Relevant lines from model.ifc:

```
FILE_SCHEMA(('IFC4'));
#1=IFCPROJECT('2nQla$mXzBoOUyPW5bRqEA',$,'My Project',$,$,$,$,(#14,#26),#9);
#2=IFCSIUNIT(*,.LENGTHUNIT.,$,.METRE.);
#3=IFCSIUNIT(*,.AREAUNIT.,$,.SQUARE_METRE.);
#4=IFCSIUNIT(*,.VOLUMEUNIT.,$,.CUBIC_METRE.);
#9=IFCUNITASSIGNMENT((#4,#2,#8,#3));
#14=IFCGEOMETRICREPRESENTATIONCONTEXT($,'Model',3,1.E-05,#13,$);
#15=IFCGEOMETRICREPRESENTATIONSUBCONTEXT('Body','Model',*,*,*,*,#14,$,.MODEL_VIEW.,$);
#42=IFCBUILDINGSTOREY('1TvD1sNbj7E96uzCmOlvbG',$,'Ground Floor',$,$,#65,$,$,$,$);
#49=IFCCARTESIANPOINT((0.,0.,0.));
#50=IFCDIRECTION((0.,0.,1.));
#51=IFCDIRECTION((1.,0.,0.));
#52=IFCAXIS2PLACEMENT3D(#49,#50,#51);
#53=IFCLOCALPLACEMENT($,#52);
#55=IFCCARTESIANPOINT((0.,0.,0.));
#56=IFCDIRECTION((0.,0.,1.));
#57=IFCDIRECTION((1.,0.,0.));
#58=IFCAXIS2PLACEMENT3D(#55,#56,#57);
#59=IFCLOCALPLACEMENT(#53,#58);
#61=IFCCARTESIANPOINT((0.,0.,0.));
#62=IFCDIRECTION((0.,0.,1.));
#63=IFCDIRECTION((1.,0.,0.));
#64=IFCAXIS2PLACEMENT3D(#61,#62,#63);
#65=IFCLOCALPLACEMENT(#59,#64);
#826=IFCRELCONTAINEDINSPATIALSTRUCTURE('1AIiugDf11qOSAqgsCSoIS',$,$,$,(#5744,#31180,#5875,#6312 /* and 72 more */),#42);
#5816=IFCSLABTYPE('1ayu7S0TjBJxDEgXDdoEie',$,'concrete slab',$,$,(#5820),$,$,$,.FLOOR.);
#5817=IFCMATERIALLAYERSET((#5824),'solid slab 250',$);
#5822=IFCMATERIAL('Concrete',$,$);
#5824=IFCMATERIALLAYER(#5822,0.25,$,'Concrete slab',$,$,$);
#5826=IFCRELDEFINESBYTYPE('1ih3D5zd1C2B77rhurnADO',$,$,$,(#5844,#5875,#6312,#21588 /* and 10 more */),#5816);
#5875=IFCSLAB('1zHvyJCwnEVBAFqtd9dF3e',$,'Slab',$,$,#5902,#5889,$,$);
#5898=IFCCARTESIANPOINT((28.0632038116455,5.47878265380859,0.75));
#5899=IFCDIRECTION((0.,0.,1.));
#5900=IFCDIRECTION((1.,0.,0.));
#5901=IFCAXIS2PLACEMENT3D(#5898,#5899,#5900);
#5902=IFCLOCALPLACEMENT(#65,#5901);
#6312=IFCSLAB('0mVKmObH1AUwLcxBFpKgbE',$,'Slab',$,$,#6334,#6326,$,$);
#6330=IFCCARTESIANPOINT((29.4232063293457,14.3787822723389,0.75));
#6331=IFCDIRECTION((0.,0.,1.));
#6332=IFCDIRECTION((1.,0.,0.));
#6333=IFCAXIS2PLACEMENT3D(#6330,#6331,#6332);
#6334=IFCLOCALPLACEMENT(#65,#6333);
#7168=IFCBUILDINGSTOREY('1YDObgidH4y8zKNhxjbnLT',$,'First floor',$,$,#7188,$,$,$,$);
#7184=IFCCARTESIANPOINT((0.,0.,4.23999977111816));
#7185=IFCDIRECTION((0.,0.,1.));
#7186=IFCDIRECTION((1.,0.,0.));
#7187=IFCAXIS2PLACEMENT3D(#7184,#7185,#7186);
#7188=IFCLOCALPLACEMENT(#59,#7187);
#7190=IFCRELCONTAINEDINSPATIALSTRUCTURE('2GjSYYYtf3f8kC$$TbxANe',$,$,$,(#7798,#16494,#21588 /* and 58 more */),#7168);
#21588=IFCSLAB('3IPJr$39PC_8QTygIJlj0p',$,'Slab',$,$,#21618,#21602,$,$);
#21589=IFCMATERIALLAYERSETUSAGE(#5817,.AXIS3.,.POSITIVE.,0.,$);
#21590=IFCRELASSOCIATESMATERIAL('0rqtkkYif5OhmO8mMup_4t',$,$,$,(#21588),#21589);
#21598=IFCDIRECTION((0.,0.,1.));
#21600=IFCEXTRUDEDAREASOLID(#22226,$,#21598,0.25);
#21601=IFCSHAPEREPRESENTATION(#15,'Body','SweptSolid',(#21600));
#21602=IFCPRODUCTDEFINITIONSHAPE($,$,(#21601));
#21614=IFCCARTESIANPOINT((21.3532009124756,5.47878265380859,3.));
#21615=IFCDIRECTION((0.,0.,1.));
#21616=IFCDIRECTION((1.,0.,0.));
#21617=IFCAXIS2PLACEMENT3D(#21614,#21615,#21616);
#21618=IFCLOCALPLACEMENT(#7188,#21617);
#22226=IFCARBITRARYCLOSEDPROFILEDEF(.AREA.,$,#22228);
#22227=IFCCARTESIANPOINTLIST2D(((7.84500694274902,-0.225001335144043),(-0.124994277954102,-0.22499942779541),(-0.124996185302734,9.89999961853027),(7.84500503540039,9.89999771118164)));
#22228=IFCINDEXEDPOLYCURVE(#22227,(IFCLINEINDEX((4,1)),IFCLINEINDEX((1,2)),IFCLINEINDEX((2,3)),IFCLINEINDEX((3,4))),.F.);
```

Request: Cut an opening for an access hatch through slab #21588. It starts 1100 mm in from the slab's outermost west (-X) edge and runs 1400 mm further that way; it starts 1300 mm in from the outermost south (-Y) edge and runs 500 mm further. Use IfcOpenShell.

```python
import numpy as np
import ifcopenshell
import ifcopenshell.api.feature
import ifcopenshell.api.geometry
import ifcopenshell.api.root
import ifcopenshell.geom
import ifcopenshell.util.placement
import ifcopenshell.util.representation
import ifcopenshell.util.shape
import ifcopenshell.util.unit

model = ifcopenshell.open("model.ifc")
unit_scale = ifcopenshell.util.unit.calculate_unit_scale(model)
settings = ifcopenshell.geom.settings()


def volume(element):
    """Net volume in cubic metres, openings subtracted."""
    shape = ifcopenshell.geom.create_shape(settings, element)
    return ifcopenshell.util.shape.get_volume(shape.geometry)


slab = model.by_guid("3IPJr$39PC_8QTygIJlj0p")
before = volume(slab)

# Extent in the slab's own axes, in metres. The edges named are its -X and -Y sides.
slab_shape = ifcopenshell.geom.create_shape(settings, slab)
vertices = ifcopenshell.util.shape.get_vertices(slab_shape.geometry)
x_min, y_min, bottom = vertices.min(axis=0)
top = vertices[:, 2].max()

opening = ifcopenshell.api.root.create_entity(model, ifc_class="IfcOpeningElement", name="Access hatch opening", predefined_type="OPENING")
context = ifcopenshell.util.representation.get_context(model, "Model", "Body", "MODEL_VIEW")
width, depth = 1.4, 0.5
outline = [(0.0, 0.0), (width, 0.0), (width, depth), (0.0, depth), (0.0, 0.0)]
# Overshoot both faces by 50 mm so the cut is clean.
shape = ifcopenshell.api.geometry.add_slab_representation(
    model, context=context, depth=top - bottom + 0.1, polyline=outline
)
ifcopenshell.api.geometry.assign_representation(model, product=opening, representation=shape)

matrix = ifcopenshell.util.placement.get_local_placement(slab.ObjectPlacement)
matrix[:, 3] = matrix @ np.append(np.array([x_min + 1.1, y_min + 1.3, bottom - 0.05]) / unit_scale, 1.0)
ifcopenshell.api.geometry.edit_object_placement(model, product=opening, matrix=matrix, is_si=False)
ifcopenshell.api.feature.add_feature(model, feature=opening, element=slab)

after = volume(slab)

print(f"slab volume {before:.3f} -> {after:.3f} m3")

model.write("model_edited.ifc")
```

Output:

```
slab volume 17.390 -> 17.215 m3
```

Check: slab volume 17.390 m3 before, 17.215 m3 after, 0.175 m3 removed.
